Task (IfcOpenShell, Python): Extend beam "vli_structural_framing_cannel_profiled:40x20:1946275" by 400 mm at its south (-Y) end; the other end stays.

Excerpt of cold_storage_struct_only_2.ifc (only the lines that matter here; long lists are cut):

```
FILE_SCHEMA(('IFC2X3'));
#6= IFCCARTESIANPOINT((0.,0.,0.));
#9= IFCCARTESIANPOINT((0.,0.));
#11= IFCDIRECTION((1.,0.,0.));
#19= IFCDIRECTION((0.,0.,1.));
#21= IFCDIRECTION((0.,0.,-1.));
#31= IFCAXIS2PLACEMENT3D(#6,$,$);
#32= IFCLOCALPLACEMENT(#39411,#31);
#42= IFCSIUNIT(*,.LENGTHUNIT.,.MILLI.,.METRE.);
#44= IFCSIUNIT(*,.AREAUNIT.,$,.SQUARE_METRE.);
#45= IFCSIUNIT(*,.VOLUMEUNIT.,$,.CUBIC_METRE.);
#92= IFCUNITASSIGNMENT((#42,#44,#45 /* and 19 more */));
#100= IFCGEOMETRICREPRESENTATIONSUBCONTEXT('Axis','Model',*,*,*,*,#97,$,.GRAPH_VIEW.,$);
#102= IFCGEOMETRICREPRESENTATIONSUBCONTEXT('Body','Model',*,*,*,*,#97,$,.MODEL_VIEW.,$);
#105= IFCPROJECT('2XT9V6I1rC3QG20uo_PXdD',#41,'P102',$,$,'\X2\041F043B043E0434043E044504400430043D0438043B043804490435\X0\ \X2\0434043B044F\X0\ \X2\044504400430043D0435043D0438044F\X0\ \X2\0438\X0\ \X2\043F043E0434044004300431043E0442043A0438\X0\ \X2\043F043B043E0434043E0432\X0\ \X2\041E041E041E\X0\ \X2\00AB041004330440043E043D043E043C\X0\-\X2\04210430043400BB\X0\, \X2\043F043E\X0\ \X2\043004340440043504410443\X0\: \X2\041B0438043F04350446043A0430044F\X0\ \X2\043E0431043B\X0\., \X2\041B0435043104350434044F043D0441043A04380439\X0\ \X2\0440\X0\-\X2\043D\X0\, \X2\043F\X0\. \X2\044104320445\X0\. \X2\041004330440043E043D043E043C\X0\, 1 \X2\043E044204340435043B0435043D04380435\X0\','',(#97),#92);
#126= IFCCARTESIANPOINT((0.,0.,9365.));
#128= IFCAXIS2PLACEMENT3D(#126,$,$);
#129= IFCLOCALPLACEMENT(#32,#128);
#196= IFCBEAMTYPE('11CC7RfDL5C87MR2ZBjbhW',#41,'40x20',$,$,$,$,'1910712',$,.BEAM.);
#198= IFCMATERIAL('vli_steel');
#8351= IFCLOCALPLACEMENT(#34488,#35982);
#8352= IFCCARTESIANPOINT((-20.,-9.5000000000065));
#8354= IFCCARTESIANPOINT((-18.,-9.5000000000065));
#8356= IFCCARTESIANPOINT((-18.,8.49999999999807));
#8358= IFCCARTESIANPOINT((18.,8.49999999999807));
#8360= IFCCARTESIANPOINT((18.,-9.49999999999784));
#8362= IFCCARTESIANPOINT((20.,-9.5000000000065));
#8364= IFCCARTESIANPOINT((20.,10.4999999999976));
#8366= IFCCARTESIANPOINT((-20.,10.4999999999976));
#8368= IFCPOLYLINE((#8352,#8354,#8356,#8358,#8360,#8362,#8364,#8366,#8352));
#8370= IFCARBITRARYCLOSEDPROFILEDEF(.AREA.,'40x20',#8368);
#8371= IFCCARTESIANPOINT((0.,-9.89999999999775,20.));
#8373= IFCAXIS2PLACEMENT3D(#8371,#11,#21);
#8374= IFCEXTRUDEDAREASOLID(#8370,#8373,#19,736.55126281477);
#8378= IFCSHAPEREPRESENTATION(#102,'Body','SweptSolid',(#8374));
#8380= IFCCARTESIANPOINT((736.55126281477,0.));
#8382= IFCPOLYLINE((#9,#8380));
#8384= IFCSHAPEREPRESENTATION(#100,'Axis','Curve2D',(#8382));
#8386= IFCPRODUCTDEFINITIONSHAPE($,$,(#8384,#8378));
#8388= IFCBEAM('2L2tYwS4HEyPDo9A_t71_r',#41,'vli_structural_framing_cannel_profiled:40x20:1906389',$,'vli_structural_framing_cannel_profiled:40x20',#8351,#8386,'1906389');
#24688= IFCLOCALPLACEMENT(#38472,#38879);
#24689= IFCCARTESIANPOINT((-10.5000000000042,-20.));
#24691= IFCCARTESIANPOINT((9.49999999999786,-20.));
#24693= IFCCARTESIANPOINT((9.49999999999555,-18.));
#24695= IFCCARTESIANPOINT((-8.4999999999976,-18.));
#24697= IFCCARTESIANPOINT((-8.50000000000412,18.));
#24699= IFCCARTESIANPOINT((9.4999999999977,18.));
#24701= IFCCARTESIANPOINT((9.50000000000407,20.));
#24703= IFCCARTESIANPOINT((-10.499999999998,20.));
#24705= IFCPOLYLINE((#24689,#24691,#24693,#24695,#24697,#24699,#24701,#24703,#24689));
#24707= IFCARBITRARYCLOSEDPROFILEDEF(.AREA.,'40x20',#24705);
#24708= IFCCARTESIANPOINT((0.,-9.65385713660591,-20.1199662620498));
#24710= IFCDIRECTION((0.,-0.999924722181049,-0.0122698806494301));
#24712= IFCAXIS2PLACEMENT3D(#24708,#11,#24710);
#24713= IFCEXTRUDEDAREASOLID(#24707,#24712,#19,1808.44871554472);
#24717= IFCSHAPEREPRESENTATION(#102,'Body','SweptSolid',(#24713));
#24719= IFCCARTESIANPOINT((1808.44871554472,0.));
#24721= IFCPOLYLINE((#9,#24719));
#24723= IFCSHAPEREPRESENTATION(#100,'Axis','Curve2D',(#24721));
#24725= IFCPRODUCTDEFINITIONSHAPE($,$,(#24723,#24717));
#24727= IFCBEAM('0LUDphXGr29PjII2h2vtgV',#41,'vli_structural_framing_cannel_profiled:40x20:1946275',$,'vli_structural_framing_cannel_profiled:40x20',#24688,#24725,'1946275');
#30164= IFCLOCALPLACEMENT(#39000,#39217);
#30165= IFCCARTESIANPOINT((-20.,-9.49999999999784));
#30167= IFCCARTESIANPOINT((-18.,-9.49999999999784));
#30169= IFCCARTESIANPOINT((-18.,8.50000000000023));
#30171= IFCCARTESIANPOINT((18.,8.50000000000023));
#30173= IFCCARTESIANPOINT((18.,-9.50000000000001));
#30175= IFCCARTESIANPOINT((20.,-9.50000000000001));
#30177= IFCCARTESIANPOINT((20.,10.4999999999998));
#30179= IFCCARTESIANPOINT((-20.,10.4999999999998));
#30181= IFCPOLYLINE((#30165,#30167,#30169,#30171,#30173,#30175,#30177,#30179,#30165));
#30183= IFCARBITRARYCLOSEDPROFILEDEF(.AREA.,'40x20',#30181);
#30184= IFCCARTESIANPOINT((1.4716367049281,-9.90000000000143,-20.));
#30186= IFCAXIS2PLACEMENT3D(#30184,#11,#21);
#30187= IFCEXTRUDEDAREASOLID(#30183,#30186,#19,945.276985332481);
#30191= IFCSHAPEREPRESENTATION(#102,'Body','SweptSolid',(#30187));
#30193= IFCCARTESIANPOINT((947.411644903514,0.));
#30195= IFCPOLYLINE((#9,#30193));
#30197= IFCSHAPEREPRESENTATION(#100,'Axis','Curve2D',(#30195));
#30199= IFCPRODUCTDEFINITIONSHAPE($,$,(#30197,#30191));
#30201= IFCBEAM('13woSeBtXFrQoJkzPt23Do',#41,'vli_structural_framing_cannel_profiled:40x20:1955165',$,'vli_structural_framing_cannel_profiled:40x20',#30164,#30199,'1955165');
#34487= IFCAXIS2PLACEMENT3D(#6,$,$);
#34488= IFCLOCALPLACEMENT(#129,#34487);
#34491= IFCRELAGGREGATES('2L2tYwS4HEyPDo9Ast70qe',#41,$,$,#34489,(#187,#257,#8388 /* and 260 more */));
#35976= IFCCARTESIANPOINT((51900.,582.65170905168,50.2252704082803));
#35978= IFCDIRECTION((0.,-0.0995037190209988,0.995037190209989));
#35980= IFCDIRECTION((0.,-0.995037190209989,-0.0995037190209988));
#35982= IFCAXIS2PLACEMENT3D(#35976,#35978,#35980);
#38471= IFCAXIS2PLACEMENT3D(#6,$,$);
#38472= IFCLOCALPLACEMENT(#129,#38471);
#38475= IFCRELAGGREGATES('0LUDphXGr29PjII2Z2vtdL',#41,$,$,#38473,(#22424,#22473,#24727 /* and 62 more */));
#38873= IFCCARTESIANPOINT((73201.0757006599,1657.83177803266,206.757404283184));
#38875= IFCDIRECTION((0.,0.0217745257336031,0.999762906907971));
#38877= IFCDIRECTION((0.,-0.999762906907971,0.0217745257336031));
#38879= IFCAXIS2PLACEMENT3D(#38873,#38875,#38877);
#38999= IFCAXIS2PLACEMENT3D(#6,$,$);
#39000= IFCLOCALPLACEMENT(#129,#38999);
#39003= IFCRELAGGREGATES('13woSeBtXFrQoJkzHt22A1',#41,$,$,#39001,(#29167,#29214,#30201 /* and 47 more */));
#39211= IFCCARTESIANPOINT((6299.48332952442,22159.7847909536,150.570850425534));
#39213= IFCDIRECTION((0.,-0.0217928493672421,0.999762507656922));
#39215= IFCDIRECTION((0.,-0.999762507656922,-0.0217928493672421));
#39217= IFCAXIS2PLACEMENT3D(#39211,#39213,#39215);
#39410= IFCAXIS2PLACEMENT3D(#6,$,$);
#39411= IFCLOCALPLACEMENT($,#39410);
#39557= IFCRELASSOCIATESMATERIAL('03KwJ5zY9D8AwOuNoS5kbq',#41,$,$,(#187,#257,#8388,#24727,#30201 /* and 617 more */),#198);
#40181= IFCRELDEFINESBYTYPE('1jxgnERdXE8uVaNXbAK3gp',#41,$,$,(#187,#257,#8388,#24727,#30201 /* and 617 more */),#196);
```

```python
import numpy as np
import ifcopenshell
import ifcopenshell.util.representation
import ifcopenshell.util.unit

model = ifcopenshell.open("cold_storage_struct_only_2.ifc")
unit_scale = ifcopenshell.util.unit.calculate_unit_scale(model)

member = model.by_id(24727)
change = 0.4 / unit_scale

# The extrusion runs towards the end named, so only its depth changes.
body = ifcopenshell.util.representation.get_representation(member, "Model", "Body")
solid = body.Items[0]
old_length = solid.Depth
solid.Depth += change

# Move the axis end point with it.
axis = next(r for r in member.Representation.Representations if r.RepresentationIdentifier == "Axis").Items[0]
start, end = (np.array(p.Coordinates) for p in axis.Points)
end = end + (end - start) / np.linalg.norm(end - start) * change
point = model.createIfcCartesianPoint(end.tolist())
axis.Points = [axis.Points[0], point]

print(f"length {old_length:g} -> {solid.Depth:g}")

model.write("cold_storage_struct_only_2_rev.ifc")
```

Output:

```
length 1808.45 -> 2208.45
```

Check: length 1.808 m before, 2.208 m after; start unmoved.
